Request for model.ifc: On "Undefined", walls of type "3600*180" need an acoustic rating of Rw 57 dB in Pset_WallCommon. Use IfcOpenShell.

First a look at what the model holds.

```python
import ifcopenshell
import ifcopenshell.util.element

model = ifcopenshell.open("model.ifc")
print(model.schema)
storey = next(s for s in model.by_type("IfcBuildingStorey") if s.Name == "Undefined")
walls = [e for e in ifcopenshell.util.element.get_decomposition(storey) if e.is_a("IfcWall")]
seen = {}
for e in walls:
    element_type = ifcopenshell.util.element.get_type(e)
    key = (element_type.Name if element_type != e and element_type else None, ifcopenshell.util.element.get_pset(e, "Pset_WallCommon", "AcousticRating"))
    seen[key] = seen.get(key, 0) + 1
for (name, value), count in sorted(seen.items(), key=str):
    print(count, "x", name, "|", value)
```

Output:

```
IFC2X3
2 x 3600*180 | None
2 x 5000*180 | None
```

```python
import ifcopenshell
import ifcopenshell.api.pset
import ifcopenshell.util.element

model = ifcopenshell.open("model.ifc")

storey = next(s for s in model.by_type("IfcBuildingStorey") if s.Name == "Undefined")
walls = [e for e in ifcopenshell.util.element.get_decomposition(storey) if e.is_a("IfcWall")]

count = 0
for e in walls:
    element_type = ifcopenshell.util.element.get_type(e)
    if element_type in (None, e) or element_type.Name != "3600*180":
        continue
    # add_pset returns the element's existing set when there is one.
    pset = ifcopenshell.api.pset.add_pset(model, product=e, name="Pset_WallCommon")
    ifcopenshell.api.pset.edit_pset(model, pset=pset, properties={"AcousticRating": "Rw 57 dB"})
    count += 1

print(count, "walls updated")

model.write("model-out.ifc")
```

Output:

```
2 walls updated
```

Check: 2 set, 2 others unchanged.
